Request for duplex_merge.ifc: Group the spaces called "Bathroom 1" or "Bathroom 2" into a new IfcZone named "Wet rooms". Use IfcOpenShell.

First a look at what the model holds.

```python
import ifcopenshell

model = ifcopenshell.open("duplex_merge.ifc")
print(model.schema)
seen = {}
for space in model.by_type("IfcSpace"):
    seen[space.LongName] = seen.get(space.LongName, 0) + 1
for name, count in sorted(seen.items(), key=str):
    print(count, "x", name)
print("zones:", [z.Name for z in model.by_type("IfcZone")][:20])
```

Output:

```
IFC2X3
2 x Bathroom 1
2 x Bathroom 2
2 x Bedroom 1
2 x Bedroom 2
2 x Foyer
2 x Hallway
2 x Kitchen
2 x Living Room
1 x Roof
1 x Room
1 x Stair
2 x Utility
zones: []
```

```python
import ifcopenshell
import ifcopenshell.api.group
import ifcopenshell.api.root

model = ifcopenshell.open("duplex_merge.ifc")

names = {"Bathroom 1", "Bathroom 2"}
spaces = [s for s in model.by_type("IfcSpace") if s.LongName in names]

zone = ifcopenshell.api.root.create_entity(model, ifc_class="IfcZone", name="Wet rooms")
ifcopenshell.api.group.assign_group(model, products=spaces, group=zone)
print(len(spaces), "spaces in", zone.Name)

model.write("duplex_merge_edited.ifc")
```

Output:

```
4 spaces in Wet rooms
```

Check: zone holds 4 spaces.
